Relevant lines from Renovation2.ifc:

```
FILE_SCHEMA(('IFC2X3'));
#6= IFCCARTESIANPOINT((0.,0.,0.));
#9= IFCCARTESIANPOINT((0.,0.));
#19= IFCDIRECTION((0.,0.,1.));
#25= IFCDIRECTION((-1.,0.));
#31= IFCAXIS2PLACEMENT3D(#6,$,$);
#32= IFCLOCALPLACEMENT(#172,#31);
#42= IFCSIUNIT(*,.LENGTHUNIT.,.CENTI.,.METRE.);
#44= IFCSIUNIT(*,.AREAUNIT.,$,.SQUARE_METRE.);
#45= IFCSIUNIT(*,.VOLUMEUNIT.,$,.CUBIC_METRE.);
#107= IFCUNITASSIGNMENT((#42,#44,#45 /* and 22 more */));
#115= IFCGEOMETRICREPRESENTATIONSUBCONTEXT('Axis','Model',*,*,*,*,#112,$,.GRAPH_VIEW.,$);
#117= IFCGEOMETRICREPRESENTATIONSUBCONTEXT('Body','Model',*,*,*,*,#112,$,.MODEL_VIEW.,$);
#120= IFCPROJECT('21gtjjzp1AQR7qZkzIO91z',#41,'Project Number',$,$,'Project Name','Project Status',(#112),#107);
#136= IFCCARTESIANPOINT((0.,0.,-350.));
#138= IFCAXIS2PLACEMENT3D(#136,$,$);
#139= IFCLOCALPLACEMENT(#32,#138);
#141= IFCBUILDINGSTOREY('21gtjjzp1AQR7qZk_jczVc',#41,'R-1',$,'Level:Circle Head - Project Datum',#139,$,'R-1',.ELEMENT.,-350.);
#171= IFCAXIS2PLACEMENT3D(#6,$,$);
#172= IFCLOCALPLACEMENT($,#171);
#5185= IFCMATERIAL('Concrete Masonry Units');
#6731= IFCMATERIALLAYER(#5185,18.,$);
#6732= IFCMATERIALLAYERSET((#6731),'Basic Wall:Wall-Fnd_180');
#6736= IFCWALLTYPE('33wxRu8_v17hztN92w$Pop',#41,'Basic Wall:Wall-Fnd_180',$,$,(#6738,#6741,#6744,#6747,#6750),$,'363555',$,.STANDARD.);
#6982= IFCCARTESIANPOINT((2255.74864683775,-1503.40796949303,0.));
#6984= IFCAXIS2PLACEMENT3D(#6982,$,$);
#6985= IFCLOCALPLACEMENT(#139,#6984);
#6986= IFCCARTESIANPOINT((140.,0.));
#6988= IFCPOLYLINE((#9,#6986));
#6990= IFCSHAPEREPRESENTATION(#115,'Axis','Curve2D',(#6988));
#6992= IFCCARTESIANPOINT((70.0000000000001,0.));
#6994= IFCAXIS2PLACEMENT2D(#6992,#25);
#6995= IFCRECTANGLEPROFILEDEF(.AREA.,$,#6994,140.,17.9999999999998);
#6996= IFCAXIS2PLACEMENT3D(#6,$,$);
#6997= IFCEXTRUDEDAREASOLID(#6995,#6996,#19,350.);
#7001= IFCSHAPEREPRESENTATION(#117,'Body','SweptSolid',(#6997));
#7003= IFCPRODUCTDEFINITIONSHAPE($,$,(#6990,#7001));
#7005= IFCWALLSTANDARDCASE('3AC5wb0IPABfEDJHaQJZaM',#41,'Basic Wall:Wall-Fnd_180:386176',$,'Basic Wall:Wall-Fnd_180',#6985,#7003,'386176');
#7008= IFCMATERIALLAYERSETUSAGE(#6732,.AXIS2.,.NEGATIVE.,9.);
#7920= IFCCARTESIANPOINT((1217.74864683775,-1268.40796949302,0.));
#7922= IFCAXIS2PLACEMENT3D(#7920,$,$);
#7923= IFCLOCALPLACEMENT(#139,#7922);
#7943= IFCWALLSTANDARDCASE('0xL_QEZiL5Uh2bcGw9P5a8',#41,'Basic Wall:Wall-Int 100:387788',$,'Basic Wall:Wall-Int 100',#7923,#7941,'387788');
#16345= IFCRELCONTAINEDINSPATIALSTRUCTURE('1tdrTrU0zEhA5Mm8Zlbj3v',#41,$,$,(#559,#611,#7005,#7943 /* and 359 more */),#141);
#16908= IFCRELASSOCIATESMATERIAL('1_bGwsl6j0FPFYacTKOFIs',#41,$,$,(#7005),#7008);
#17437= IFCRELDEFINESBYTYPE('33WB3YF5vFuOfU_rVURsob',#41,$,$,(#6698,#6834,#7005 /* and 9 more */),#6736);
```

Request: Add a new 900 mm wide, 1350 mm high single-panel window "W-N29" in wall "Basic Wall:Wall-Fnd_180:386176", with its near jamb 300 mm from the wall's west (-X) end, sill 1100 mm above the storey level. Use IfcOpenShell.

```python
import numpy as np
import ifcopenshell
import ifcopenshell.api.feature
import ifcopenshell.api.geometry
import ifcopenshell.api.root
import ifcopenshell.api.spatial
import ifcopenshell.api.type
import ifcopenshell.geom
import ifcopenshell.util.element
import ifcopenshell.util.placement
import ifcopenshell.util.representation
import ifcopenshell.util.shape
import ifcopenshell.util.unit

model = ifcopenshell.open("Renovation2.ifc")
unit_scale = ifcopenshell.util.unit.calculate_unit_scale(model)
settings = ifcopenshell.geom.settings()


def volume(element):
    """Net volume in cubic metres, openings subtracted."""
    shape = ifcopenshell.geom.create_shape(settings, element)
    return ifcopenshell.util.shape.get_volume(shape.geometry)


wall = model.by_guid("3AC5wb0IPABfEDJHaQJZaM")
storey = ifcopenshell.util.element.get_container(wall, ifc_class="IfcBuildingStorey")
context = ifcopenshell.util.representation.get_context(model, "Model", "Body", "MODEL_VIEW")
before = volume(wall)

width, height, from_end, sill = 0.9, 1.35, 0.3, 1.1  # metres

# The wall runs along its own X axis, and the end named is its -X end.
wall_shape = ifcopenshell.geom.create_shape(settings, wall)
x, y, z = ifcopenshell.util.shape.get_vertices(wall_shape.geometry).T
start = x.min() + from_end
face, thickness = float(y.min()), float(y.max() - y.min())
wall_matrix = ifcopenshell.util.placement.get_local_placement(wall.ObjectPlacement)
level = ifcopenshell.util.placement.get_local_placement(storey.ObjectPlacement)[2, 3]


def in_wall(x, y):
    """Placement at x, y metres in the wall's axes, at sill height."""
    matrix = wall_matrix.copy()
    matrix[:, 3] = wall_matrix @ np.array([x / unit_scale, y / unit_scale, 0.0, 1.0])
    matrix[2, 3] = level + sill / unit_scale
    return matrix


# Opening: a box that overshoots both wall faces by 50 mm.
opening = ifcopenshell.api.root.create_entity(model, ifc_class="IfcOpeningElement")
box = ifcopenshell.api.geometry.add_wall_representation(
    model, context=context, length=width, height=height, thickness=thickness + 0.1
)
ifcopenshell.api.geometry.assign_representation(model, product=opening, representation=box)
ifcopenshell.api.geometry.edit_object_placement(model, product=opening, matrix=in_wall(start, face - 0.05), is_si=False)
ifcopenshell.api.feature.add_feature(model, feature=opening, element=wall)

window = ifcopenshell.api.root.create_entity(model, ifc_class="IfcWindow", name="W-N29")
window.OverallWidth, window.OverallHeight = width / unit_scale, height / unit_scale
body = ifcopenshell.api.geometry.add_window_representation(
    model,
    context=context,
    overall_width=window.OverallWidth,
    overall_height=window.OverallHeight,
    partition_type="SINGLE_PANEL",
)
ifcopenshell.api.geometry.assign_representation(model, product=window, representation=body)
ifcopenshell.api.spatial.assign_container(model, products=[window], relating_structure=storey)
fills = ifcopenshell.api.feature.add_filling(model, opening=opening, element=window)
fills.OwnerHistory = window.OwnerHistory  # required in IFC2X3

# IFC2X3 keeps the operation on the window style.
style = ifcopenshell.api.root.create_entity(model, ifc_class="IfcWindowStyle", name="W-N29")
style.OperationType, style.ConstructionType = "SINGLE_PANEL", "NOTDEFINED"
style.ParameterTakesPrecedence = style.Sizeable = False
ifcopenshell.api.type.assign_type(model, related_objects=[window], relating_type=style)

# Centre the window in the wall's thickness.
ifcopenshell.api.geometry.edit_object_placement(model, product=window, matrix=in_wall(start, face), is_si=False)
window_shape = ifcopenshell.geom.create_shape(settings, window)
depth = ifcopenshell.util.shape.get_vertices(window_shape.geometry)[:, 1]
offset = face + thickness / 2 - (depth.min() + depth.max()) / 2
ifcopenshell.api.geometry.edit_object_placement(model, product=window, matrix=in_wall(start, offset), is_si=False)

after = volume(wall)

print(f"wall volume {before:.3f} -> {after:.3f} m3")

model.write("Renovation2_v2.ifc")
```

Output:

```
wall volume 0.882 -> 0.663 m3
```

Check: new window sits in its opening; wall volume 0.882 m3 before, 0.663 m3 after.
